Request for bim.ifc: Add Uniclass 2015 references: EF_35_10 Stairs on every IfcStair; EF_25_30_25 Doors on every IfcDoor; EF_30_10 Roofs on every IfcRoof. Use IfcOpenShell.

First a look at what the model holds.

```python
import ifcopenshell

model = ifcopenshell.open("bim.ifc")
print(model.schema)
print("classifications:", [c.Name for c in model.by_type("IfcClassification")])
for ifc_class in ("IfcDoor", "IfcRoof", "IfcStair", "IfcWall", "IfcWindow"):
    print(ifc_class, len(model.by_type(ifc_class)))
```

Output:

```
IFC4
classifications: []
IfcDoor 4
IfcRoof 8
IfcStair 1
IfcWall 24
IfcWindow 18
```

```python
import ifcopenshell
import ifcopenshell.api.classification

model = ifcopenshell.open("bim.ifc")

system = ifcopenshell.api.classification.add_classification(model, classification="Uniclass 2015")

codes = {
    "IfcStair": ("EF_35_10", "Stairs"),
    "IfcDoor": ("EF_25_30_25", "Doors"),
    "IfcRoof": ("EF_30_10", "Roofs"),
}
for ifc_class, (code, name) in codes.items():
    products = model.by_type(ifc_class)
    ifcopenshell.api.classification.add_reference(
        model, products=products, classification=system, identification=code, name=name
    )
    print(code, len(products))

model.write("bim-out.ifc")
```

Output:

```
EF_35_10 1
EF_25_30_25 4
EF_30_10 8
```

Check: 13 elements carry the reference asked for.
